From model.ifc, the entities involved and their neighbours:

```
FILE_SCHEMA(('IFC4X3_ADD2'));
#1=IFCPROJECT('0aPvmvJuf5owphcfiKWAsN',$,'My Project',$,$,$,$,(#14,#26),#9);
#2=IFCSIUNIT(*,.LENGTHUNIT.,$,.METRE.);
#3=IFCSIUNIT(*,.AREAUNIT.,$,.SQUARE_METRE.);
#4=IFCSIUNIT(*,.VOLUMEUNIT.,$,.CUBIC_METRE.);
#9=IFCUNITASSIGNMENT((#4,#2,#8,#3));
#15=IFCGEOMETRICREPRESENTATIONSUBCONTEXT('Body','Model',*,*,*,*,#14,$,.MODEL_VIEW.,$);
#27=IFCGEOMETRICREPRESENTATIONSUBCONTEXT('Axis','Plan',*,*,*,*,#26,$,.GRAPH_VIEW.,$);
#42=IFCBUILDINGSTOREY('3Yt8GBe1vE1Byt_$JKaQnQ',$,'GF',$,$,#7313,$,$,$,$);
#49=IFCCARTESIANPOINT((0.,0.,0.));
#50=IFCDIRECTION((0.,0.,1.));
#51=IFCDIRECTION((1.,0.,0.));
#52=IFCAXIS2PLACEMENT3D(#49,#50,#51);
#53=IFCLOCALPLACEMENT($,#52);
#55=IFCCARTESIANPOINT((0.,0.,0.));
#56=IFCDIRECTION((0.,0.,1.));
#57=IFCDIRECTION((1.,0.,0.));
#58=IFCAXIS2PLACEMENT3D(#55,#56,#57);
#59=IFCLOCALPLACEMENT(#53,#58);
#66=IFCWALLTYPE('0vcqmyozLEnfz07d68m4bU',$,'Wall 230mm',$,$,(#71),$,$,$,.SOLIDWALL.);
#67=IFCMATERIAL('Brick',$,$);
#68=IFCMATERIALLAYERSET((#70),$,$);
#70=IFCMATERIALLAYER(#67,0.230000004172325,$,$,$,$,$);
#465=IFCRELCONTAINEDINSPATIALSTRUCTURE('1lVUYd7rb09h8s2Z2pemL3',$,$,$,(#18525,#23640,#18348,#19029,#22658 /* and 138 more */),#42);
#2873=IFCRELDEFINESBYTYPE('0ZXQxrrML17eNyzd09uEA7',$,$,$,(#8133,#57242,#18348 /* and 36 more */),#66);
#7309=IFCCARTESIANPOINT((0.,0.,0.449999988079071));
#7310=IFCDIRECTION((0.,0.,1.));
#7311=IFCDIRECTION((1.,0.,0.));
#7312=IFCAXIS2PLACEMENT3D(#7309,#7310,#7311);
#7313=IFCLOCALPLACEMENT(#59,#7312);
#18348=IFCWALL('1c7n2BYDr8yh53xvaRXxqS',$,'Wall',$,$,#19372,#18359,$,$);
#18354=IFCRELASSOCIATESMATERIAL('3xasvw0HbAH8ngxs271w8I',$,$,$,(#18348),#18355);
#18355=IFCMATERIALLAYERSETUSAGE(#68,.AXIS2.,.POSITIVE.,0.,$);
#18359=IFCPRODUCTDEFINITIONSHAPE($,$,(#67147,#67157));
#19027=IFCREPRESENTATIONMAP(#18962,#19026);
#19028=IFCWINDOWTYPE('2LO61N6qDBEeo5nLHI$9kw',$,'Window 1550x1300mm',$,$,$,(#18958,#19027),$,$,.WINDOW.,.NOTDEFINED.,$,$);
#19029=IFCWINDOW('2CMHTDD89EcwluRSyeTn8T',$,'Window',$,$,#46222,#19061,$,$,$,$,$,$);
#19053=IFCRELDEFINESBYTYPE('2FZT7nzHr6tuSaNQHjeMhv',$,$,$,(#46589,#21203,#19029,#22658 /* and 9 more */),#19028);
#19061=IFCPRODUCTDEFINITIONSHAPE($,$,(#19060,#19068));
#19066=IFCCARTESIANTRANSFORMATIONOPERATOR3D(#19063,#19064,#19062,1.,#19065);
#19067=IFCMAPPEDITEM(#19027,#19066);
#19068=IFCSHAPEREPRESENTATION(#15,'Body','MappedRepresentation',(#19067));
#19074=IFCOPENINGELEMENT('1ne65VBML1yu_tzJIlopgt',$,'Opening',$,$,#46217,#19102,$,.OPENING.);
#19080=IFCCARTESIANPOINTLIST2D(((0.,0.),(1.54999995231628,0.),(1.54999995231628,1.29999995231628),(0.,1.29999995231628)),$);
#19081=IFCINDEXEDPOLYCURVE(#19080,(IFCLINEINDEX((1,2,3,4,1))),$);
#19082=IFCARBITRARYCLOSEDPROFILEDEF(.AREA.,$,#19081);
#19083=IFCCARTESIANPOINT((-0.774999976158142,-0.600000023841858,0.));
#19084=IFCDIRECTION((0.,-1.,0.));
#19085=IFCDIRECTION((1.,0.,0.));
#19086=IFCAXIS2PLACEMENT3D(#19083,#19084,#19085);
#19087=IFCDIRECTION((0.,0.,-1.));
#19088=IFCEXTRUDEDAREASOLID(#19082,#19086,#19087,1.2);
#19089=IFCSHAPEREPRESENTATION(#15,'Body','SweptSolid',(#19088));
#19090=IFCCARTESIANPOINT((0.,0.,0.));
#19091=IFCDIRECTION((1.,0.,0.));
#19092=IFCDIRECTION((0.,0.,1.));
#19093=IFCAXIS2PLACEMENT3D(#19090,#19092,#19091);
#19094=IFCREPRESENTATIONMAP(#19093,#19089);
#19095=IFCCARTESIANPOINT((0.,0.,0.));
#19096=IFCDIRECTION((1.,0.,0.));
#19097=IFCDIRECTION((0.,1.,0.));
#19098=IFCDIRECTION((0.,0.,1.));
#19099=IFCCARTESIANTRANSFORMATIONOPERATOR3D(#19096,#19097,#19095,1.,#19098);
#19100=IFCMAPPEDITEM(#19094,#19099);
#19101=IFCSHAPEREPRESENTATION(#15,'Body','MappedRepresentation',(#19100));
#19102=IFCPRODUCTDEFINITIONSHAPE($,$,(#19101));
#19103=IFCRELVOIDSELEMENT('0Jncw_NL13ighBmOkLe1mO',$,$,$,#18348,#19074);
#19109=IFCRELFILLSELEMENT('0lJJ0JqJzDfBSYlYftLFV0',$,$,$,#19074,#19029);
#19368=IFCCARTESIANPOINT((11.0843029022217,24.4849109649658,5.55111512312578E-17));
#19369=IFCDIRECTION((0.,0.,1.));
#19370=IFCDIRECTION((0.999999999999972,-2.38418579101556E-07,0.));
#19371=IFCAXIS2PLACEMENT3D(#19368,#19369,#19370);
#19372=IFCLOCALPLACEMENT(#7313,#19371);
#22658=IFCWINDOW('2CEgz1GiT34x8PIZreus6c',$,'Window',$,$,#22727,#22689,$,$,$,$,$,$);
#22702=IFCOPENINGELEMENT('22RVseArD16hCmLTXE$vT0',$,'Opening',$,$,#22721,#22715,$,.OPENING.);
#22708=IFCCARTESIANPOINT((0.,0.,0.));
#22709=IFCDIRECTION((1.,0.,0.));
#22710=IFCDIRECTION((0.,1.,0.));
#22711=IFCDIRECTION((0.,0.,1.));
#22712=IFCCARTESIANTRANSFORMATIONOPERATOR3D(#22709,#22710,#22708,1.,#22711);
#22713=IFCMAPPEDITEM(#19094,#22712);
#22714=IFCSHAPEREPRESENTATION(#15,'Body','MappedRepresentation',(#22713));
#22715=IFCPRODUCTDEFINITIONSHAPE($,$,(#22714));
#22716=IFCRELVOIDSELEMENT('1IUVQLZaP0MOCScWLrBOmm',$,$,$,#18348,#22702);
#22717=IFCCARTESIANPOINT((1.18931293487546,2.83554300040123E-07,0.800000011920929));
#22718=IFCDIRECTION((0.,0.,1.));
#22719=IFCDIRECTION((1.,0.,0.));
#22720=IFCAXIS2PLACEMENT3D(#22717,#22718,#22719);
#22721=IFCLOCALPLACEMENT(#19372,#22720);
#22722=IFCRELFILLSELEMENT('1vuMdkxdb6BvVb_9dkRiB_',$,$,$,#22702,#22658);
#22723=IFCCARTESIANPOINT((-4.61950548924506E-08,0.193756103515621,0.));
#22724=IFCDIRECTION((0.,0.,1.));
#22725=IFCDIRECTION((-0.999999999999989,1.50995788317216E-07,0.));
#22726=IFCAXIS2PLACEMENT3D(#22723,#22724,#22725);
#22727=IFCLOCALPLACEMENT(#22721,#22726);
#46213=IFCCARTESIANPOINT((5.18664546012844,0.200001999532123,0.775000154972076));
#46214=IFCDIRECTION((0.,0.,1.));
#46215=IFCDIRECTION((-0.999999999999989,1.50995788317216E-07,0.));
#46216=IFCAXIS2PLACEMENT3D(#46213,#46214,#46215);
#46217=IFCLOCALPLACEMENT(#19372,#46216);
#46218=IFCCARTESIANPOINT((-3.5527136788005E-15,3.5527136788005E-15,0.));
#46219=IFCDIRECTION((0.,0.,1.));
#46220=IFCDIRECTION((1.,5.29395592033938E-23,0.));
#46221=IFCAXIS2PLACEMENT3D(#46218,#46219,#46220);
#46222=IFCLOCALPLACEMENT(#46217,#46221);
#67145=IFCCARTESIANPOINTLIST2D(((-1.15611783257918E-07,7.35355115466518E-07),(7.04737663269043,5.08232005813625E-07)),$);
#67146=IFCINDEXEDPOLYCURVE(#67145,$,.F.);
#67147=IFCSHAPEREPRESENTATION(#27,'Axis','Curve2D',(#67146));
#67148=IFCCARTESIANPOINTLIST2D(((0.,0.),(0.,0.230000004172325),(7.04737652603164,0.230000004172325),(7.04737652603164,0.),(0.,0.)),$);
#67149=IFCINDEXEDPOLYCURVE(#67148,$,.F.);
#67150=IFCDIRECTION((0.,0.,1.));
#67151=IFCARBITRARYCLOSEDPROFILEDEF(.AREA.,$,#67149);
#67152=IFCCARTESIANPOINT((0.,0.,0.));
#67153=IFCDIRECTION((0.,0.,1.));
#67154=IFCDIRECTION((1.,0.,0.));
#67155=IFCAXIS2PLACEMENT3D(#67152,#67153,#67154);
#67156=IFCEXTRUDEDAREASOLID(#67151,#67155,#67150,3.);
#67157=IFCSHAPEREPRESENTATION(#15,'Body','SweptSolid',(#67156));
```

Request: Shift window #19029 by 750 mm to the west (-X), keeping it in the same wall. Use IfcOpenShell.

```python
import ifcopenshell
import ifcopenshell.api.geometry
import ifcopenshell.util.placement

model = ifcopenshell.open("model.ifc")

window = model.by_guid("2CMHTDD89EcwluRSyeTn8T")
opening = window.FillsVoids[0].RelatingOpeningElement
wall = opening.VoidsElements[0].RelatingBuildingElement

wall_matrix = ifcopenshell.util.placement.get_local_placement(wall.ObjectPlacement)
shift = wall_matrix[:3, 0] * -0.75
before = ifcopenshell.util.placement.get_local_placement(window.ObjectPlacement)[:3, 3].copy()

# The window is placed relative to its opening, so it follows when the opening moves.
matrix = ifcopenshell.util.placement.get_local_placement(opening.ObjectPlacement)
matrix[:3, 3] += shift
ifcopenshell.api.geometry.edit_object_placement(
    model, product=opening, matrix=matrix, is_si=False, should_transform_children=True
)

after = ifcopenshell.util.placement.get_local_placement(window.ObjectPlacement)[:3, 3]
print("window moved by", (after - before).round(3) + 0.0)

model.write("model_rev.ifc")
```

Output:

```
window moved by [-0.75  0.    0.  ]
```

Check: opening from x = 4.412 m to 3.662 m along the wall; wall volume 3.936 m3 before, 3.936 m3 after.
